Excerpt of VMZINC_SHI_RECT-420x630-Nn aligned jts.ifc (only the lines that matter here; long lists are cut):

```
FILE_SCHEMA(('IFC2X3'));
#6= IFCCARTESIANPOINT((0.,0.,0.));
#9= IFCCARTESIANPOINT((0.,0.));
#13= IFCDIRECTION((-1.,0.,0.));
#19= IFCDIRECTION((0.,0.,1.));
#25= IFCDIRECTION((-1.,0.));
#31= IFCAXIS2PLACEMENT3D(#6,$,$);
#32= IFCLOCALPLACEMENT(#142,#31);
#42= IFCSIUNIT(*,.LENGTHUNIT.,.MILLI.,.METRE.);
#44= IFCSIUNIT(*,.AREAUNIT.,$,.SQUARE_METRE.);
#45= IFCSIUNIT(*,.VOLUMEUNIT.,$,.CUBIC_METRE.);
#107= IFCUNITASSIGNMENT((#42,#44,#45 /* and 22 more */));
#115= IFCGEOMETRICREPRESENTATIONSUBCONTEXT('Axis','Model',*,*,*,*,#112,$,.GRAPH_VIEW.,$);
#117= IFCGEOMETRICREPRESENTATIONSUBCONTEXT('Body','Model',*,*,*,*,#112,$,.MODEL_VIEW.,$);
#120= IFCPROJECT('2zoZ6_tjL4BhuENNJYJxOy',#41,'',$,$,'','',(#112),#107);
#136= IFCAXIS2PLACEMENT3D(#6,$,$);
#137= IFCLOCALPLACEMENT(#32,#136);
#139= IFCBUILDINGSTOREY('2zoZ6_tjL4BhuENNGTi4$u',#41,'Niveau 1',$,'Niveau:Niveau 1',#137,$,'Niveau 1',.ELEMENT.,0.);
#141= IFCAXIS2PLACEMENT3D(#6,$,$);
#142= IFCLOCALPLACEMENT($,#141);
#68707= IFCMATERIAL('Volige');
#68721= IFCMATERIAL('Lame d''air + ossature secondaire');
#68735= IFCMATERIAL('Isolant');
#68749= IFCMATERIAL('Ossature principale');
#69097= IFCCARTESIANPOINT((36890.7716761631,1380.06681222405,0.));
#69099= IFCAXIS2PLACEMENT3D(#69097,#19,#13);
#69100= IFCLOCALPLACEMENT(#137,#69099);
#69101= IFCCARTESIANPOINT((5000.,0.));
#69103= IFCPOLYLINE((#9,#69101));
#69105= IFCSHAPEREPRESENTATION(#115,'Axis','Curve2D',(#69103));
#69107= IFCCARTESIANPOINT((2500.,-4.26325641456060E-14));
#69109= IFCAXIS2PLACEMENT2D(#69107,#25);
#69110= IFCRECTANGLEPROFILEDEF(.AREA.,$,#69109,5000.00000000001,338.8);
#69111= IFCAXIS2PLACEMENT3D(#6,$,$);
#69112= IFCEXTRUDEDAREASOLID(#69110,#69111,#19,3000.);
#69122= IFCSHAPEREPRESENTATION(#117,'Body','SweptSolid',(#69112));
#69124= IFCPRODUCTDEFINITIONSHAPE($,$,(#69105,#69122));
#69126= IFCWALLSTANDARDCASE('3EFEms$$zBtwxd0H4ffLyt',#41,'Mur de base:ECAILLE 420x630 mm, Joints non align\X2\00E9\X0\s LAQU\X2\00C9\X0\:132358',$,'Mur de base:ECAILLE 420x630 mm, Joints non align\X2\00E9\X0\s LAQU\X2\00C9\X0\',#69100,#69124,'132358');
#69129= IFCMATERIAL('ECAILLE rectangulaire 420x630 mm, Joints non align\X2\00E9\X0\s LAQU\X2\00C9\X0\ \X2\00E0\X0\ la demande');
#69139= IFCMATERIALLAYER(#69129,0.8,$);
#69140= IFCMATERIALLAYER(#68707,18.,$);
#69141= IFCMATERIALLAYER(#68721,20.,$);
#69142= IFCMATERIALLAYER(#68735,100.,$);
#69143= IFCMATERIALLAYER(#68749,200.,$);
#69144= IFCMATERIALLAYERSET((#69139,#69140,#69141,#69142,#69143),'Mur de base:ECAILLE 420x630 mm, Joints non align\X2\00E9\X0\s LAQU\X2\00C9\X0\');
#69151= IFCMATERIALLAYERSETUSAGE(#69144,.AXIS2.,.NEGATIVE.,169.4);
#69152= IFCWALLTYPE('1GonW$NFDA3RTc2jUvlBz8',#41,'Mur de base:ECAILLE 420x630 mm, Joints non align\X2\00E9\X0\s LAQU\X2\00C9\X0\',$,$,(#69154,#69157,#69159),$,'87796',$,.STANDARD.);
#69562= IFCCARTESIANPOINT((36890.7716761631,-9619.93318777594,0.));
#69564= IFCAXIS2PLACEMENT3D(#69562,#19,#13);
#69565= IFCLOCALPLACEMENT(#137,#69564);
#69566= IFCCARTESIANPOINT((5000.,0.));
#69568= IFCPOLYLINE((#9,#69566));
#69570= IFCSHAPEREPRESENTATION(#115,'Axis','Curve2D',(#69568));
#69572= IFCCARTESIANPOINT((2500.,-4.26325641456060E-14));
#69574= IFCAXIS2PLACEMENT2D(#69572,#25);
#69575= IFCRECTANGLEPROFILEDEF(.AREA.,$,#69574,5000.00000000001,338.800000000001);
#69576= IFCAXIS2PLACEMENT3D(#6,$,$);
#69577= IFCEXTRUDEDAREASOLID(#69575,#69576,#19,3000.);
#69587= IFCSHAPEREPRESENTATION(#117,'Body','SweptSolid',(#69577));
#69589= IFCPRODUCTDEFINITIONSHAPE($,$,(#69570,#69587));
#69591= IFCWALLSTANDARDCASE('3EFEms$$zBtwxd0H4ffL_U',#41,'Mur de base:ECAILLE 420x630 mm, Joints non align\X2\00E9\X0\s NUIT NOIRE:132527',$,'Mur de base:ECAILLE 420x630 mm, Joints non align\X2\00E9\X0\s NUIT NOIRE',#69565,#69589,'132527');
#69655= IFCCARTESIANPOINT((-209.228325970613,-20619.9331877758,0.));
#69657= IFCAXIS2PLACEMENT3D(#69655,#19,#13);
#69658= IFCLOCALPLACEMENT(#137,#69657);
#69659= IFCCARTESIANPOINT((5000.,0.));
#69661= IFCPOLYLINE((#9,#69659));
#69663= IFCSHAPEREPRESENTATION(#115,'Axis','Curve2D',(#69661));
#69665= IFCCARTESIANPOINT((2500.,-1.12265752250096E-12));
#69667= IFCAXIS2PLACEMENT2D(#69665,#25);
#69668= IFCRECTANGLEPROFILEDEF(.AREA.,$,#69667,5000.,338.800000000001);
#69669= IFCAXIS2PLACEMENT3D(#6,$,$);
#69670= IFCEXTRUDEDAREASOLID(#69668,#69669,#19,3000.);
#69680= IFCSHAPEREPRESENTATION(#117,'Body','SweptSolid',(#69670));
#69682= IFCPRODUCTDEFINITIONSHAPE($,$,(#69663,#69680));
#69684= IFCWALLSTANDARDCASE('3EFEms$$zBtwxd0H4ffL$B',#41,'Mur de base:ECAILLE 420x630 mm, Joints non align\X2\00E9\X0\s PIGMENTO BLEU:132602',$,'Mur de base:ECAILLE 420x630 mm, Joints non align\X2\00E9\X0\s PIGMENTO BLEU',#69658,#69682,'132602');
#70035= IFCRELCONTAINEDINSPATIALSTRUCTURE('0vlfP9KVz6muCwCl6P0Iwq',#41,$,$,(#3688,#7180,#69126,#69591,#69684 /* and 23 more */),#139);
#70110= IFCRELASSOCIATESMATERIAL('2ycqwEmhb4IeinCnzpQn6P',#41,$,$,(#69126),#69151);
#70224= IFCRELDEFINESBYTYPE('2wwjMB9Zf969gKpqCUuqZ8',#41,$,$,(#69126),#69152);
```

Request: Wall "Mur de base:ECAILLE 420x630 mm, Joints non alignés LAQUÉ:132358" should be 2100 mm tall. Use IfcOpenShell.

```python
import ifcopenshell
import ifcopenshell.geom
import ifcopenshell.util.representation
import ifcopenshell.util.shape
import ifcopenshell.util.unit

model = ifcopenshell.open("VMZINC_SHI_RECT-420x630-Nn aligned jts.ifc")
unit_scale = ifcopenshell.util.unit.calculate_unit_scale(model)
settings = ifcopenshell.geom.settings()


def volume(element):
    """Net volume in cubic metres, openings subtracted."""
    shape = ifcopenshell.geom.create_shape(settings, element)
    return ifcopenshell.util.shape.get_volume(shape.geometry)


wall = model.by_id(69126)
before = volume(wall)

body = ifcopenshell.util.representation.get_representation(wall, "Model", "Body")
solid = body.Items[0]
old_height = solid.Depth
solid.Depth = 2.1 / unit_scale
after = volume(wall)

print(f"height {old_height:g} -> {solid.Depth:g}, volume {before:.3f} -> {after:.3f} m3")

model.write("VMZINC_SHI_RECT-420x630-Nn aligned jts_edited.ifc")
```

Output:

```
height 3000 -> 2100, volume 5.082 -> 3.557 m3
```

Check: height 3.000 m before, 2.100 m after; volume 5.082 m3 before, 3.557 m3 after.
